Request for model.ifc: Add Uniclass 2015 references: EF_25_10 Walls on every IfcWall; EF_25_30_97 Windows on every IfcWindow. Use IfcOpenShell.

First a look at what the model holds.

```python
import ifcopenshell

model = ifcopenshell.open("model.ifc")
print(model.schema)
print("classifications:", [c.Name for c in model.by_type("IfcClassification")])
for ifc_class in ("IfcDoor", "IfcRoof", "IfcStair", "IfcWall", "IfcWindow"):
    print(ifc_class, len(model.by_type(ifc_class)))
```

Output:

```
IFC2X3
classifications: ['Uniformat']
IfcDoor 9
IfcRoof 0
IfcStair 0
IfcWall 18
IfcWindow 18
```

```python
import ifcopenshell
import ifcopenshell.api.classification

model = ifcopenshell.open("model.ifc")

# IFC2X3 requires Source and Edition and has no link from the project to the system.
system = model.create_entity("IfcClassification", Source="NBS", Edition="2015", Name="Uniclass 2015")

codes = {
    "IfcWall": ("EF_25_10", "Walls"),
    "IfcWindow": ("EF_25_30_97", "Windows"),
}
for ifc_class, (code, name) in codes.items():
    products = model.by_type(ifc_class)
    ifcopenshell.api.classification.add_reference(
        model, products=products, classification=system, identification=code, name=name
    )
    print(code, len(products))

model.write("model-out.ifc")
```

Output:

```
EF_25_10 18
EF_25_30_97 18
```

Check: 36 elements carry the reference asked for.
